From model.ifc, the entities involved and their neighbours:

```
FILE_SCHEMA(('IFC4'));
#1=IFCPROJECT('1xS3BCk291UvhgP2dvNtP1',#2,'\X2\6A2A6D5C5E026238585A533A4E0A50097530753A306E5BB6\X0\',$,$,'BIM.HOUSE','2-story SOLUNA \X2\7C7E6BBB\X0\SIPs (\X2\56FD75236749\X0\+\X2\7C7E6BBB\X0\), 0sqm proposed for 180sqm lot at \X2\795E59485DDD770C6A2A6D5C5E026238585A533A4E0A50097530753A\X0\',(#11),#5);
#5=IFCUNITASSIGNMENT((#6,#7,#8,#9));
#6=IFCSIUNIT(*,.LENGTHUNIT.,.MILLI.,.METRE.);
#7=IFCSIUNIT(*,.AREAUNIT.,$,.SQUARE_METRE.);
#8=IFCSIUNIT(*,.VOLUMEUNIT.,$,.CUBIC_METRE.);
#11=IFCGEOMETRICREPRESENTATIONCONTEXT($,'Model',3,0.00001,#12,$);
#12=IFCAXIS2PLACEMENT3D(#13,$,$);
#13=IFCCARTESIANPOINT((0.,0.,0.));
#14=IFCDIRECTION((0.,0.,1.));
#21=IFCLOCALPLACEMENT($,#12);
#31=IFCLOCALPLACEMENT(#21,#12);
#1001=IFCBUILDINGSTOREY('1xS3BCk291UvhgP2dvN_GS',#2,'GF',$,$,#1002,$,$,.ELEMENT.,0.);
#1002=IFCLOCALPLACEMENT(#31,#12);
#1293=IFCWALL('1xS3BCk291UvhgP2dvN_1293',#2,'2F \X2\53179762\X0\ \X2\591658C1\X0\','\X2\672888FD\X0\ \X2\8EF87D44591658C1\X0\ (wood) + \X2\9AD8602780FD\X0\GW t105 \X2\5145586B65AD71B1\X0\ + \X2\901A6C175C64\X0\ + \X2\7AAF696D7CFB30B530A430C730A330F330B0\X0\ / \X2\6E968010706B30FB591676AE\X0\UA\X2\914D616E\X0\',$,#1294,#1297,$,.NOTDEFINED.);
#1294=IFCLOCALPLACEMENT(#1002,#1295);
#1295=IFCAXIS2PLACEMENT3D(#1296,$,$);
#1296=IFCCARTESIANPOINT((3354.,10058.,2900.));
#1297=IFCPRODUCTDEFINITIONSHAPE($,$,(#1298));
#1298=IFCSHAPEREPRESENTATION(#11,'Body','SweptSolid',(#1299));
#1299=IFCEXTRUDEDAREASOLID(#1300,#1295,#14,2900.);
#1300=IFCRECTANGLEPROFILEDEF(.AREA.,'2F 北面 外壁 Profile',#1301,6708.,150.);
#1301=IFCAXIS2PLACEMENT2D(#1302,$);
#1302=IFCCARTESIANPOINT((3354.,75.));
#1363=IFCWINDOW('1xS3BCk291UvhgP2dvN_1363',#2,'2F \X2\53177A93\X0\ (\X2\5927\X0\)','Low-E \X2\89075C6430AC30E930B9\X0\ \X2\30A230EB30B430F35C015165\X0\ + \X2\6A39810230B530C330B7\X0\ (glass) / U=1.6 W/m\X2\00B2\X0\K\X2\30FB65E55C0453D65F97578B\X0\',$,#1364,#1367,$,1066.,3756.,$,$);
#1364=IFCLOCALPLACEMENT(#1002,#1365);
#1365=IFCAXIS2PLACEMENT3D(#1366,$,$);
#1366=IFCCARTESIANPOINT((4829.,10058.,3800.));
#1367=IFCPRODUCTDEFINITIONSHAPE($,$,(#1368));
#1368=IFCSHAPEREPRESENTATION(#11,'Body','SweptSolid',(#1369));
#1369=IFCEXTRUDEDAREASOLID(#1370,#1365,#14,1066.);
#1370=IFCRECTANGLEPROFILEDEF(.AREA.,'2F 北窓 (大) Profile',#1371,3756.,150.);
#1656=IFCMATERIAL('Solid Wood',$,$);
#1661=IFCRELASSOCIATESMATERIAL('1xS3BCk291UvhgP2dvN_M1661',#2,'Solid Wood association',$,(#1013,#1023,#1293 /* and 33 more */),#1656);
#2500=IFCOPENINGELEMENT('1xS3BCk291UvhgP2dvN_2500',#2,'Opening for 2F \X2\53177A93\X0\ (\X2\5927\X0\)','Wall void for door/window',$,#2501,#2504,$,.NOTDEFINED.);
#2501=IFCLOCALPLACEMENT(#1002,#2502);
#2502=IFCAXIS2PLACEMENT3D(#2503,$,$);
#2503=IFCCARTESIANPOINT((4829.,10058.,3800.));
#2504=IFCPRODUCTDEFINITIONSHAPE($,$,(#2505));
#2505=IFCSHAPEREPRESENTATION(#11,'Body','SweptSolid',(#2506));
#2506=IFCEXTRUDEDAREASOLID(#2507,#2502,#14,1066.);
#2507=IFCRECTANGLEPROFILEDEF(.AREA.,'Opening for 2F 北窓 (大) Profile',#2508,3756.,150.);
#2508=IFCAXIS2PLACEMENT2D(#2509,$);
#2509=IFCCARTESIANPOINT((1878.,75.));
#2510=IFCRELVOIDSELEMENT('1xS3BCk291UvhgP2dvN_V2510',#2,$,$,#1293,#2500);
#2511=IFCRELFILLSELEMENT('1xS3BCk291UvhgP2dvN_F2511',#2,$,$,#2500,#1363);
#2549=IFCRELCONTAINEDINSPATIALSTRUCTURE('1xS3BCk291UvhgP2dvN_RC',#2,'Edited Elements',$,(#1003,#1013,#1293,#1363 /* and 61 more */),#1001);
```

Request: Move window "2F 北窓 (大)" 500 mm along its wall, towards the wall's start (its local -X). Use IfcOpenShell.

```python
import ifcopenshell
import ifcopenshell.api.geometry
import ifcopenshell.util.placement
import ifcopenshell.util.unit

model = ifcopenshell.open("model.ifc")
unit_scale = ifcopenshell.util.unit.calculate_unit_scale(model)

window = model.by_guid("1xS3BCk291UvhgP2dvN_1363")
opening = window.FillsVoids[0].RelatingOpeningElement
wall = opening.VoidsElements[0].RelatingBuildingElement

wall_matrix = ifcopenshell.util.placement.get_local_placement(wall.ObjectPlacement)
shift = wall_matrix[:3, 0] * -0.5 / unit_scale
before = ifcopenshell.util.placement.get_local_placement(window.ObjectPlacement)[:3, 3].copy()

# The window is not placed relative to its opening, so move both.
for product in (opening, window):
    matrix = ifcopenshell.util.placement.get_local_placement(product.ObjectPlacement)
    matrix[:3, 3] += shift
    ifcopenshell.api.geometry.edit_object_placement(model, product=product, matrix=matrix, is_si=False)

after = ifcopenshell.util.placement.get_local_placement(window.ObjectPlacement)[:3, 3]
print("window moved by", (after - before).round(3) + 0.0)

model.write("model_v2.ifc")
```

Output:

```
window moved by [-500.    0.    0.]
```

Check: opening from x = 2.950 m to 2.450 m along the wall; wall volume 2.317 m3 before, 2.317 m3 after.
